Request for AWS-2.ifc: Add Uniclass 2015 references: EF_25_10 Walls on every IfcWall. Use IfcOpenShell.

First a look at what the model holds.

```python
import ifcopenshell

model = ifcopenshell.open("AWS-2.ifc")
print(model.schema)
print("classifications:", [c.Name for c in model.by_type("IfcClassification")])
for ifc_class in ("IfcDoor", "IfcRoof", "IfcStair", "IfcWall", "IfcWindow"):
    print(ifc_class, len(model.by_type(ifc_class)))
```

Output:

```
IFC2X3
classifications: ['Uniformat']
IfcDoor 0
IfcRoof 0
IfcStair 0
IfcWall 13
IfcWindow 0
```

```python
import ifcopenshell
import ifcopenshell.api.classification

model = ifcopenshell.open("AWS-2.ifc")

# IFC2X3 requires Source and Edition and has no link from the project to the system.
system = model.create_entity("IfcClassification", Source="NBS", Edition="2015", Name="Uniclass 2015")

codes = {
    "IfcWall": ("EF_25_10", "Walls"),
}
for ifc_class, (code, name) in codes.items():
    products = model.by_type(ifc_class)
    ifcopenshell.api.classification.add_reference(
        model, products=products, classification=system, identification=code, name=name
    )
    print(code, len(products))

model.write("AWS-2_updated.ifc")
```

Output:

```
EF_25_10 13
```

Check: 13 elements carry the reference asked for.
